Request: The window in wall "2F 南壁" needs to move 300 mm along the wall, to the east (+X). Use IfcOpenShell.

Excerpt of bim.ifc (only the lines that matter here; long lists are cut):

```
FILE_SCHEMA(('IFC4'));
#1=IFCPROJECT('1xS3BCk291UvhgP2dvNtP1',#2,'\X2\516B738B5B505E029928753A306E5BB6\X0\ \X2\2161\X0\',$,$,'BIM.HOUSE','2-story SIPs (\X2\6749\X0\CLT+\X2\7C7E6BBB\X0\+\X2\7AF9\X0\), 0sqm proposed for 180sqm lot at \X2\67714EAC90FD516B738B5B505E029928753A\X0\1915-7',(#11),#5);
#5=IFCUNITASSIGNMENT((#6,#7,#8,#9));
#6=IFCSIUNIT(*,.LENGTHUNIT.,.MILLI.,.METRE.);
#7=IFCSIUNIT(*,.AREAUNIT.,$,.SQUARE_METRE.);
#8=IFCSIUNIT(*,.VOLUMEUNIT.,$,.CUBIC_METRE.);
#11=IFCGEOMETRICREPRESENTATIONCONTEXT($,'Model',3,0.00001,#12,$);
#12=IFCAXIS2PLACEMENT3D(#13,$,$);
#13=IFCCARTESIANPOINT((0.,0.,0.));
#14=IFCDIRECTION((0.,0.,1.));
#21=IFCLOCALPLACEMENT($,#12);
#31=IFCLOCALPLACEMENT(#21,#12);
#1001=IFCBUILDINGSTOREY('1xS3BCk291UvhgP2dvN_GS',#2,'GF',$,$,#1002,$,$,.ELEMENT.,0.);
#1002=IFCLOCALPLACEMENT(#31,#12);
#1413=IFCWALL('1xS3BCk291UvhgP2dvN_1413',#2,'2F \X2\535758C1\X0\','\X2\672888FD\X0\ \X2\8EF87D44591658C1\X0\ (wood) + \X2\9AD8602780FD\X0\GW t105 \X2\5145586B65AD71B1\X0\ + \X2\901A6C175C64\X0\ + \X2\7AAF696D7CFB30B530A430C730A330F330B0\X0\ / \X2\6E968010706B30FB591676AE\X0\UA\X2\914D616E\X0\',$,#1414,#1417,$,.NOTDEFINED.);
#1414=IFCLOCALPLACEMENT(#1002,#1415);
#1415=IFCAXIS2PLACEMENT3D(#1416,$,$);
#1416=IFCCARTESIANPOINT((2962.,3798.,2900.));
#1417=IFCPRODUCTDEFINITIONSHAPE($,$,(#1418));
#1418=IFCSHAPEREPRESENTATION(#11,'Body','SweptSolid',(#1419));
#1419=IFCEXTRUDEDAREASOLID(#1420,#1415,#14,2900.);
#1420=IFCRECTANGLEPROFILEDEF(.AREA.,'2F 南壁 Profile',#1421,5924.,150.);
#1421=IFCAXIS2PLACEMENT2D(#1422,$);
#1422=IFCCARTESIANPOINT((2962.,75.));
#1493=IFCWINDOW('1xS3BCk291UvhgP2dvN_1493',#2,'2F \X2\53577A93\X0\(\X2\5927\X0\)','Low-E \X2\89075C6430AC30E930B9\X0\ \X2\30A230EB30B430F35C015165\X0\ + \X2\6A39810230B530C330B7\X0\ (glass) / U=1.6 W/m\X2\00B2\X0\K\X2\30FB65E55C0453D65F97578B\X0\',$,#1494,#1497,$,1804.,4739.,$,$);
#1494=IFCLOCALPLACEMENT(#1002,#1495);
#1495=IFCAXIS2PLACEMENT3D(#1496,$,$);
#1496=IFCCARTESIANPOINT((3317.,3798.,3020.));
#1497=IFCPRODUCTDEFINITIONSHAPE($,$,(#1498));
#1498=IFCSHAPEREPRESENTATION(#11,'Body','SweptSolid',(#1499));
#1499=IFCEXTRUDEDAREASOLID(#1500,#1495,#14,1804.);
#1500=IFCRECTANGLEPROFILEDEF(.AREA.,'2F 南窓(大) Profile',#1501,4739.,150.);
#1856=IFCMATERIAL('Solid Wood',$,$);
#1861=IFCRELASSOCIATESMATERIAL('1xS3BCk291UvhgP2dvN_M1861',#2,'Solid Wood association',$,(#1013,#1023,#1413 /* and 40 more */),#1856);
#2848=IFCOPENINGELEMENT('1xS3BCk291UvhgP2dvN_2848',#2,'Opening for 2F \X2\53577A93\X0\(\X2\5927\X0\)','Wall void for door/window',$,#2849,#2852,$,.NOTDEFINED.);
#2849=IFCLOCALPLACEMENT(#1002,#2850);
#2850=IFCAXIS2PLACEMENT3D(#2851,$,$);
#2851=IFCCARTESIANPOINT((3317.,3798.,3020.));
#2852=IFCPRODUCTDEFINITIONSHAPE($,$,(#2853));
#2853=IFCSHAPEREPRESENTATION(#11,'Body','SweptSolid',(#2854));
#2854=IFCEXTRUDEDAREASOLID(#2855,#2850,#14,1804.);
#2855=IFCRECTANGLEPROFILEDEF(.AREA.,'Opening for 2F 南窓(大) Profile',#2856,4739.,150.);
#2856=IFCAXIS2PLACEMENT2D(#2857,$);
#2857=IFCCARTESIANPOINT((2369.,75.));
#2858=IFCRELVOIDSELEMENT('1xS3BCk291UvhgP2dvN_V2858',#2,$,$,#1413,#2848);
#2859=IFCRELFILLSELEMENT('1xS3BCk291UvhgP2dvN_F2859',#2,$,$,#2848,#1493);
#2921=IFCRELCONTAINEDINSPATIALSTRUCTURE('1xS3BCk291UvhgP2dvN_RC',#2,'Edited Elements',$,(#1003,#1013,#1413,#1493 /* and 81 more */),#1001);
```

```python
import ifcopenshell
import ifcopenshell.api.geometry
import ifcopenshell.util.placement
import ifcopenshell.util.unit

model = ifcopenshell.open("bim.ifc")
unit_scale = ifcopenshell.util.unit.calculate_unit_scale(model)

window = model.by_guid("1xS3BCk291UvhgP2dvN_1493")
opening = window.FillsVoids[0].RelatingOpeningElement
wall = opening.VoidsElements[0].RelatingBuildingElement

wall_matrix = ifcopenshell.util.placement.get_local_placement(wall.ObjectPlacement)
shift = wall_matrix[:3, 0] * 0.3 / unit_scale
before = ifcopenshell.util.placement.get_local_placement(window.ObjectPlacement)[:3, 3].copy()

# The window is not placed relative to its opening, so move both.
for product in (opening, window):
    matrix = ifcopenshell.util.placement.get_local_placement(product.ObjectPlacement)
    matrix[:3, 3] += shift
    ifcopenshell.api.geometry.edit_object_placement(model, product=product, matrix=matrix, is_si=False)

after = ifcopenshell.util.placement.get_local_placement(window.ObjectPlacement)[:3, 3]
print("window moved by", (after - before).round(3) + 0.0)

model.write("bim_edited.ifc")
```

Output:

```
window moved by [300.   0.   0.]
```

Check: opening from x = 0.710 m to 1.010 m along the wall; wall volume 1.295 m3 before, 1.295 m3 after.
